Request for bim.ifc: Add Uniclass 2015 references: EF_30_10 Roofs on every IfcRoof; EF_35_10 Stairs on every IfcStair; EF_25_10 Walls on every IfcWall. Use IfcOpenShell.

First a look at what the model holds.

```python
import ifcopenshell

model = ifcopenshell.open("bim.ifc")
print(model.schema)
print("classifications:", [c.Name for c in model.by_type("IfcClassification")])
for ifc_class in ("IfcDoor", "IfcRoof", "IfcStair", "IfcWall", "IfcWindow"):
    print(ifc_class, len(model.by_type(ifc_class)))
```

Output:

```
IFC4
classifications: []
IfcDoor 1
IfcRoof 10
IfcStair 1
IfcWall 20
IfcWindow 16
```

```python
import ifcopenshell
import ifcopenshell.api.classification

model = ifcopenshell.open("bim.ifc")

system = ifcopenshell.api.classification.add_classification(model, classification="Uniclass 2015")

codes = {
    "IfcRoof": ("EF_30_10", "Roofs"),
    "IfcStair": ("EF_35_10", "Stairs"),
    "IfcWall": ("EF_25_10", "Walls"),
}
for ifc_class, (code, name) in codes.items():
    products = model.by_type(ifc_class)
    ifcopenshell.api.classification.add_reference(
        model, products=products, classification=system, identification=code, name=name
    )
    print(code, len(products))

model.write("bim_v2.ifc")
```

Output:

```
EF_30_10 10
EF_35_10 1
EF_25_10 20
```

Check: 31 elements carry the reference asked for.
